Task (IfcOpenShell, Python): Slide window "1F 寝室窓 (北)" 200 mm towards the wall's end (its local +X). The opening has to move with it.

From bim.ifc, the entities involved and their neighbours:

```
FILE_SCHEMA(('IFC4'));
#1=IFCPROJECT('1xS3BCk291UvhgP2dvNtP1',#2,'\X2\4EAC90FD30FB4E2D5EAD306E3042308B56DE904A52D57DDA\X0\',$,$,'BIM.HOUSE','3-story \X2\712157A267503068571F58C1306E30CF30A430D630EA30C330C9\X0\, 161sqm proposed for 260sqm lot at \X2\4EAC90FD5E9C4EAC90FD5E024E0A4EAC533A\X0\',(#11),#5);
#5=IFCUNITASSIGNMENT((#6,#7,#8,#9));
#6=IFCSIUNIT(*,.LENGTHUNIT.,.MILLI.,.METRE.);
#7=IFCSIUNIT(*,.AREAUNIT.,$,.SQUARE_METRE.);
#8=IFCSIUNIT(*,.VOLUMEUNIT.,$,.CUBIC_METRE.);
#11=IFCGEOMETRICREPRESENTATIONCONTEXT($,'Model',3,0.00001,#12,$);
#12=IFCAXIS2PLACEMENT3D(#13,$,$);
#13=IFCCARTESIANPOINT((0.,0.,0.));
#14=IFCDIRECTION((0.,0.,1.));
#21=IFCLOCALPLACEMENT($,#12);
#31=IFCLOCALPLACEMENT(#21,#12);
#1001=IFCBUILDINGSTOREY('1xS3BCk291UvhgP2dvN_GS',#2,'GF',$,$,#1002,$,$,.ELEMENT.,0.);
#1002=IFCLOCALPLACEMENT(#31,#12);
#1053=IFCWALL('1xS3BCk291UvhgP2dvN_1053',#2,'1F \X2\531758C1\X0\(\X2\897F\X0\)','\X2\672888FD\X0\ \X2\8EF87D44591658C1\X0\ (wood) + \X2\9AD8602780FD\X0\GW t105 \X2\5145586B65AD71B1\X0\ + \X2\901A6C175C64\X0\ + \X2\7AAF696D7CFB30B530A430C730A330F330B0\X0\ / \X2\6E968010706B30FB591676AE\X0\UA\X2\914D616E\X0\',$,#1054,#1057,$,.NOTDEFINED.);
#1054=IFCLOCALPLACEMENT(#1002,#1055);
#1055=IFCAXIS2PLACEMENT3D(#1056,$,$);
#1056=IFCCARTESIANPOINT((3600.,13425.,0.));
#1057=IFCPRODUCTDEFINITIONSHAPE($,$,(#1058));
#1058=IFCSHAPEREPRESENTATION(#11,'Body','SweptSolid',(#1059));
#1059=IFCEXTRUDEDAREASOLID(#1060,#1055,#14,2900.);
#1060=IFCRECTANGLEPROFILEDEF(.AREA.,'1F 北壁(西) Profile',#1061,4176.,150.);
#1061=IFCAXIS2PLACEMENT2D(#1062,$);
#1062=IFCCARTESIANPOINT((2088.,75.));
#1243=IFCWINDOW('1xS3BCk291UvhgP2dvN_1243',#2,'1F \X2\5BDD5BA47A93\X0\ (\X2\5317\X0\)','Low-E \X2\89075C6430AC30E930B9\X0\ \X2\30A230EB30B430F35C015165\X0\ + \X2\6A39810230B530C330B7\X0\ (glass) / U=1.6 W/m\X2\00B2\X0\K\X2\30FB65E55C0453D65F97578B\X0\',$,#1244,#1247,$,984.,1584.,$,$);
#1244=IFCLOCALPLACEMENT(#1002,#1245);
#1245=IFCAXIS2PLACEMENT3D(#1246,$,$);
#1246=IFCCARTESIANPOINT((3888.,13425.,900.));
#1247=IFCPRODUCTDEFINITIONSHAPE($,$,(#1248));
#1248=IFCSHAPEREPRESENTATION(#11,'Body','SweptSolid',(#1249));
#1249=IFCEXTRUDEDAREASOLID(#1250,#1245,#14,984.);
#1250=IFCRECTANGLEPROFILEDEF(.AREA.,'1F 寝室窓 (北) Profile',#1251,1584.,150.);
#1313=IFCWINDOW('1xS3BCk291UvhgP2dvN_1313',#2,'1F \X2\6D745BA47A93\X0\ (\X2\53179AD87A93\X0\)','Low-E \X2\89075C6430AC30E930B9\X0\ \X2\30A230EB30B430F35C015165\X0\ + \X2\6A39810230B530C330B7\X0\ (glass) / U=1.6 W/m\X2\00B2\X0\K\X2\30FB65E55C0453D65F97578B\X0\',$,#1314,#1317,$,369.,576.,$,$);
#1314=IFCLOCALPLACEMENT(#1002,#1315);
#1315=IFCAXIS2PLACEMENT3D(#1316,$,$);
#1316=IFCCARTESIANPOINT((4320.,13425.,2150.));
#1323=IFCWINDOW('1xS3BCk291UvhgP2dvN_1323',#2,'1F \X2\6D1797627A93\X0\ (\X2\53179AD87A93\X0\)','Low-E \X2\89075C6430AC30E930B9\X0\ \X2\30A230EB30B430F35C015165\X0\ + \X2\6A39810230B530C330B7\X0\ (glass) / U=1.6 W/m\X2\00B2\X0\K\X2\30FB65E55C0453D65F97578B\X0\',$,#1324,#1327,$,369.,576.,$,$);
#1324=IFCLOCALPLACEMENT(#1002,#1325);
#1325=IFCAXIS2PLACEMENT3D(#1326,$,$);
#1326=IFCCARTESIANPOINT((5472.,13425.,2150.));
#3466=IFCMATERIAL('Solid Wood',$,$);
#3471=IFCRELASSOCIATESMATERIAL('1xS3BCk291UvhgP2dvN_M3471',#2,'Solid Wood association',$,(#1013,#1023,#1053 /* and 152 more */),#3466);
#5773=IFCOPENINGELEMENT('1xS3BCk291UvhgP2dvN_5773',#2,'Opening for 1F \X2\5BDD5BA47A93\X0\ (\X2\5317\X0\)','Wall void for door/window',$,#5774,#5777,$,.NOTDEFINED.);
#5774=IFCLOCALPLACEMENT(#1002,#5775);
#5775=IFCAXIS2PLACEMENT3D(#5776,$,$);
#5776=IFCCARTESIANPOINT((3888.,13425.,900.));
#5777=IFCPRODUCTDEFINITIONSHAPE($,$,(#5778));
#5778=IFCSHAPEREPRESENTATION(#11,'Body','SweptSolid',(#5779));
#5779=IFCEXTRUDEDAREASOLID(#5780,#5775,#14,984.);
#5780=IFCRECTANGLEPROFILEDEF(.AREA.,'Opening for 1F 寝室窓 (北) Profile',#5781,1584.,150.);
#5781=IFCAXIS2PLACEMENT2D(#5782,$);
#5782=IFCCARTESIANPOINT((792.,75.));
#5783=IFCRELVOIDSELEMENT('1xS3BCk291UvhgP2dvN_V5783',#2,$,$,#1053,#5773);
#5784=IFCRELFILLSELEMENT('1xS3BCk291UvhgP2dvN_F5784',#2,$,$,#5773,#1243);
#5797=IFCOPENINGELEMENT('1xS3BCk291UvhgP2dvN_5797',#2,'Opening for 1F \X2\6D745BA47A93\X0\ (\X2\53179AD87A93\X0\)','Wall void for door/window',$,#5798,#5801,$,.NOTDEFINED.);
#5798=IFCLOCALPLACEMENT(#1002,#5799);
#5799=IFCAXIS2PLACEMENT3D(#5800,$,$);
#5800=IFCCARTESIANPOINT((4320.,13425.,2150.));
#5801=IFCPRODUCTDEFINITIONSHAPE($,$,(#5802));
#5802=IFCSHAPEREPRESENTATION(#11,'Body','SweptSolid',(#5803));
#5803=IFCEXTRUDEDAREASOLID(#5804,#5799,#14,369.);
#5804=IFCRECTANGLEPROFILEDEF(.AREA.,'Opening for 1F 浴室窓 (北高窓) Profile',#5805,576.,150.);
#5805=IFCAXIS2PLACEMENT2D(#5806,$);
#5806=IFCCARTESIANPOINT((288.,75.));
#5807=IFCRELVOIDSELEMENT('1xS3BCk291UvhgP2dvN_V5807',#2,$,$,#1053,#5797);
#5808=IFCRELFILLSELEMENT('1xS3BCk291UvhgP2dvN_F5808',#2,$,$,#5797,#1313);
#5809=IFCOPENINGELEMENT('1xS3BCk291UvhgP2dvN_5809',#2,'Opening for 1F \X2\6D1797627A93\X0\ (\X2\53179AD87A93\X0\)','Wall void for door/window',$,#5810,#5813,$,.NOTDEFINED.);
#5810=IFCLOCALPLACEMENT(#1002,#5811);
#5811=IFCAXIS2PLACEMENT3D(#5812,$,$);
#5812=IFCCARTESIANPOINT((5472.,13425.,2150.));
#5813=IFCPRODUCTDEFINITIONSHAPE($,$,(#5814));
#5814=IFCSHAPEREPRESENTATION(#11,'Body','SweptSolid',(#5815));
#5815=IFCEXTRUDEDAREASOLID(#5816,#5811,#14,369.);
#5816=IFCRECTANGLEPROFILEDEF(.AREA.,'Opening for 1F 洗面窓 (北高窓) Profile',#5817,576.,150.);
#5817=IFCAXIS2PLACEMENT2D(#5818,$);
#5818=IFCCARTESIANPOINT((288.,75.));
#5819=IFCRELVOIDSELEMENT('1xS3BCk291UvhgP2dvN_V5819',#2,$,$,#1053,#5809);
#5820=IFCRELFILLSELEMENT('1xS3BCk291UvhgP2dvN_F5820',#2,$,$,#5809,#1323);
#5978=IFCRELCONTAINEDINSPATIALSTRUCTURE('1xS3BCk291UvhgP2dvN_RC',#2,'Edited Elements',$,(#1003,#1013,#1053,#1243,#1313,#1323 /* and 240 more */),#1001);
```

```python
import ifcopenshell
import ifcopenshell.api.geometry
import ifcopenshell.util.placement

model = ifcopenshell.open("bim.ifc")

window = model.by_guid("1xS3BCk291UvhgP2dvN_1243")
opening = window.FillsVoids[0].RelatingOpeningElement
wall = opening.VoidsElements[0].RelatingBuildingElement

wall_matrix = ifcopenshell.util.placement.get_local_placement(wall.ObjectPlacement)
shift = wall_matrix[:3, 0] * 200.0
before = ifcopenshell.util.placement.get_local_placement(window.ObjectPlacement)[:3, 3].copy()

# The window is not placed relative to its opening, so move both.
for product in (opening, window):
    matrix = ifcopenshell.util.placement.get_local_placement(product.ObjectPlacement)
    matrix[:3, 3] += shift
    ifcopenshell.api.geometry.edit_object_placement(model, product=product, matrix=matrix, is_si=False)

after = ifcopenshell.util.placement.get_local_placement(window.ObjectPlacement)[:3, 3]
print("window moved by", (after - before).round(3) + 0.0)

model.write("bim_updated.ifc")
```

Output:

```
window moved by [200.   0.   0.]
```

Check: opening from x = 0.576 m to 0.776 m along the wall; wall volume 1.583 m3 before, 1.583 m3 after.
